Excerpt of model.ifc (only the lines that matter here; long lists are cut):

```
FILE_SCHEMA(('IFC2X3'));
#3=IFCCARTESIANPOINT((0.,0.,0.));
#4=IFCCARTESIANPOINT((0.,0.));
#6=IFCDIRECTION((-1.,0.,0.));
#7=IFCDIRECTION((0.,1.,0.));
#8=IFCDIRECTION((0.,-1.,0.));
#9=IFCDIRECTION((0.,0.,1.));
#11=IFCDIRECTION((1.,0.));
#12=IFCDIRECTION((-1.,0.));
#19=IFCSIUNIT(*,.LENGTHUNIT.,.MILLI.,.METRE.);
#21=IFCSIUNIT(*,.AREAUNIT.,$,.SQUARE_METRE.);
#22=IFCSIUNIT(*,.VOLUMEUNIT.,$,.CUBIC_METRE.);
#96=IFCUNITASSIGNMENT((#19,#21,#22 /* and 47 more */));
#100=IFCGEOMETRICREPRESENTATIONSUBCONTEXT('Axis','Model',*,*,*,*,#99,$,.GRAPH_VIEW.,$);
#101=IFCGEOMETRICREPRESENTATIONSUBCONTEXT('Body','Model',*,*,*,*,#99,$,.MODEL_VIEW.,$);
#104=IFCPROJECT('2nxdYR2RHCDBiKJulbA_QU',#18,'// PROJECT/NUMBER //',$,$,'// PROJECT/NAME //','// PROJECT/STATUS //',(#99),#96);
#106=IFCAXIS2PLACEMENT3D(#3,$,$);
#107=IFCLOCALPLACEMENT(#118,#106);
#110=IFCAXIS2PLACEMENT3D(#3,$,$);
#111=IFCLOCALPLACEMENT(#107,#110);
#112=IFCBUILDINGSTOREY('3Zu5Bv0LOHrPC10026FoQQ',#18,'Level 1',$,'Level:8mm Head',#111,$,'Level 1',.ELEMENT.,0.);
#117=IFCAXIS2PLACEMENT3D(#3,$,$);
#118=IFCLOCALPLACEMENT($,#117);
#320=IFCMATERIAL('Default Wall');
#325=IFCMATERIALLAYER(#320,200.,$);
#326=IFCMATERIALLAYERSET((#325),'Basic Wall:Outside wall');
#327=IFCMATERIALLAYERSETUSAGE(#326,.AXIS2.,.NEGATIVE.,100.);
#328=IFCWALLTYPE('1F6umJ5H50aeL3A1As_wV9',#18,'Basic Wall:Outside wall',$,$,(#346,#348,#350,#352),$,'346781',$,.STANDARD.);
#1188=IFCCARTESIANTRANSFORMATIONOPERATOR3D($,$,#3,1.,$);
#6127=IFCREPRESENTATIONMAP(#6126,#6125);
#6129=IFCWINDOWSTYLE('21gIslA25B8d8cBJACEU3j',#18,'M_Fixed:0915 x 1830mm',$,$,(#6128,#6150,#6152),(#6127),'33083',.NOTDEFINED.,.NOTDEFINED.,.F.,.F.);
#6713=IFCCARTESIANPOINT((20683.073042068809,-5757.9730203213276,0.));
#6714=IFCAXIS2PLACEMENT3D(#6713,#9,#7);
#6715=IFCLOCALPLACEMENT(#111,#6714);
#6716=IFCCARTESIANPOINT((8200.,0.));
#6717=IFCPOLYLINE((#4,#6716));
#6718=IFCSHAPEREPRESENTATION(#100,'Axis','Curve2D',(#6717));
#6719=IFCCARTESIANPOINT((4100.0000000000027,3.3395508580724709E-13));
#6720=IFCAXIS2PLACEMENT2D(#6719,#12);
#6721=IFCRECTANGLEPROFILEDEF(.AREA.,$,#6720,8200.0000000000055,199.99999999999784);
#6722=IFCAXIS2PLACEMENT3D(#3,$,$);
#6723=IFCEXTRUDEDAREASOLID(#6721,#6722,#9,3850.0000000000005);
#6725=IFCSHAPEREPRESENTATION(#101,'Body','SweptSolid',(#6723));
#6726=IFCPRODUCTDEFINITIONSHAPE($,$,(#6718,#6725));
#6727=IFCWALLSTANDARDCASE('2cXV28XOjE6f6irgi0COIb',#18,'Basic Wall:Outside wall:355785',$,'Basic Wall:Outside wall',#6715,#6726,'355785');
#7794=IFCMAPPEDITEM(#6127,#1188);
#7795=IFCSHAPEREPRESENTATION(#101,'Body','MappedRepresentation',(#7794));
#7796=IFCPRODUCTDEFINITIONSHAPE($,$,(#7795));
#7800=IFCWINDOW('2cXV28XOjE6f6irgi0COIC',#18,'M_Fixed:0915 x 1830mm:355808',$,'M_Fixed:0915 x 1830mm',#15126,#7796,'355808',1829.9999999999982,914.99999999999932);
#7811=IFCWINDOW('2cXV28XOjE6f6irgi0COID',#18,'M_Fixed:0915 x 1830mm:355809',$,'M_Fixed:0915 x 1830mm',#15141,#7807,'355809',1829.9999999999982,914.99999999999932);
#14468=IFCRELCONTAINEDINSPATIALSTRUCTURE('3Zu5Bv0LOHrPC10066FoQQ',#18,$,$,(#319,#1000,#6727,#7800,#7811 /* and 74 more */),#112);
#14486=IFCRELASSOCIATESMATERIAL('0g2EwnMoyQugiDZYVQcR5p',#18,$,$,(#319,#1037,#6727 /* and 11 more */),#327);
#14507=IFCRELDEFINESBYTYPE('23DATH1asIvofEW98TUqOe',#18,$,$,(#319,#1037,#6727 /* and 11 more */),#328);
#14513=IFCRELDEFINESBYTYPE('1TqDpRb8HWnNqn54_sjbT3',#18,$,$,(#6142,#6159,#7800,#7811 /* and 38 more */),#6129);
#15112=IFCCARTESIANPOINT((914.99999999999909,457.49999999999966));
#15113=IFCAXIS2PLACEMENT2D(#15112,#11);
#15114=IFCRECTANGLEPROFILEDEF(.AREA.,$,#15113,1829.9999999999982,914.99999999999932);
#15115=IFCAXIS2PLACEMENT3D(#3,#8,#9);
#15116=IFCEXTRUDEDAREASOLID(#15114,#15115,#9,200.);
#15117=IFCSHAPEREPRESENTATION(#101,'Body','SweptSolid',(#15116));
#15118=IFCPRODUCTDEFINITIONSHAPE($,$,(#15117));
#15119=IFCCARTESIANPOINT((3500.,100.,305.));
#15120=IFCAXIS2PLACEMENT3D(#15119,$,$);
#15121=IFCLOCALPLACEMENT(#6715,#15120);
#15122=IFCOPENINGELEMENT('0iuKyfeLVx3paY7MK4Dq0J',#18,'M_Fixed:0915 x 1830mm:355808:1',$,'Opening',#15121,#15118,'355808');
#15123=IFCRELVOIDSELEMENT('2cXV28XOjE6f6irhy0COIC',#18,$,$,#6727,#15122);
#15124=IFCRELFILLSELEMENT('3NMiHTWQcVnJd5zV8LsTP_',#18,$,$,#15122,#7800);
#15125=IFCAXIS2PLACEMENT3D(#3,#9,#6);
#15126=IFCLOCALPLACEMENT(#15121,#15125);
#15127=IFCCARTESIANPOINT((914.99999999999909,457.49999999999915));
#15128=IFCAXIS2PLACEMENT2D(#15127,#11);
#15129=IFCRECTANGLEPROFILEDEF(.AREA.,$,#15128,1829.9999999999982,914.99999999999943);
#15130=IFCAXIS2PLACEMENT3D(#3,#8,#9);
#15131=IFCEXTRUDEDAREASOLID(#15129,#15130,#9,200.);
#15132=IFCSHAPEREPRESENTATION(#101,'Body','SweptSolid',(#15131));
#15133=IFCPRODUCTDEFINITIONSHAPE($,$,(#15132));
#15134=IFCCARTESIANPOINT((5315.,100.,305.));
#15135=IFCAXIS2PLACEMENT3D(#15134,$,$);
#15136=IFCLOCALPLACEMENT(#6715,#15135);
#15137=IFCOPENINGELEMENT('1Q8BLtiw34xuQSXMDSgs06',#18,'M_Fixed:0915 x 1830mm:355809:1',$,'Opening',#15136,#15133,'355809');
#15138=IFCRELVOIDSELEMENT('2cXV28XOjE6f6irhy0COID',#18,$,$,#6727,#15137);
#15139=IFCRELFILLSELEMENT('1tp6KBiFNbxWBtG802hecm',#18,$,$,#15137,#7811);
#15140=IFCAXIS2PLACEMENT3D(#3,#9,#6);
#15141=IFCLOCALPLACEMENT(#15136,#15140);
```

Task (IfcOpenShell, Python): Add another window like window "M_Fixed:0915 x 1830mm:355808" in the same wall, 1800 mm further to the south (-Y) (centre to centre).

```python
import ifcopenshell
import ifcopenshell.api.feature
import ifcopenshell.api.geometry
import ifcopenshell.api.root
import ifcopenshell.geom
import ifcopenshell.util.element
import ifcopenshell.util.placement
import ifcopenshell.util.shape
import ifcopenshell.util.unit

model = ifcopenshell.open("model.ifc")
unit_scale = ifcopenshell.util.unit.calculate_unit_scale(model)
settings = ifcopenshell.geom.settings()


def volume(element):
    """Net volume in cubic metres, openings subtracted."""
    shape = ifcopenshell.geom.create_shape(settings, element)
    return ifcopenshell.util.shape.get_volume(shape.geometry)


def reuse_history(source, copy):
    """copy_class also copies each property set's owner history, people and application; keep the originals."""
    for rel in copy.IsDefinedBy:
        if rel.is_a("IfcRelDefinesByProperties") and (history := rel.RelatingPropertyDefinition.OwnerHistory):
            rel.RelatingPropertyDefinition.OwnerHistory = source.OwnerHistory
            ifcopenshell.util.element.remove_deep2(model, history)


window = model.by_guid("2cXV28XOjE6f6irgi0COIC")
opening = window.FillsVoids[0].RelatingOpeningElement
wall = opening.VoidsElements[0].RelatingBuildingElement
before = volume(wall)
shift = ifcopenshell.util.placement.get_local_placement(wall.ObjectPlacement)[:3, 0] * -1.8 / unit_scale

# copy_class copies the void relationship, type, container and properties, but no geometry.
new_opening = ifcopenshell.api.root.copy_class(model, product=opening)
new_opening.Representation = ifcopenshell.util.element.copy_deep(
    model, opening.Representation, exclude=["IfcGeometricRepresentationContext", "IfcRepresentationMap"]
)
new_opening.Name = "M_Fixed:0915 x 1830mm"
new_opening.Tag = None
new_window = ifcopenshell.api.root.copy_class(model, product=window)
new_window.Representation = ifcopenshell.util.element.copy_deep(
    model, window.Representation, exclude=["IfcGeometricRepresentationContext", "IfcRepresentationMap"]
)
new_window.Name = "M_Fixed:0915 x 1830mm"
new_window.Tag = None
reuse_history(window, new_window)
fills = ifcopenshell.api.feature.add_filling(model, opening=new_opening, element=new_window)
fills.OwnerHistory = new_window.OwnerHistory  # required in IFC2X3

for old, new in ((opening, new_opening), (window, new_window)):
    matrix = ifcopenshell.util.placement.get_local_placement(old.ObjectPlacement)
    matrix[:3, 3] += shift
    ifcopenshell.api.geometry.edit_object_placement(model, product=new, matrix=matrix, is_si=False)

after = volume(wall)

print(f"wall volume {before:.3f} -> {after:.3f} m3")

model.write("model_edited.ifc")
```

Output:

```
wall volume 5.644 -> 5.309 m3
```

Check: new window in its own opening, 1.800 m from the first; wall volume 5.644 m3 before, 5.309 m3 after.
